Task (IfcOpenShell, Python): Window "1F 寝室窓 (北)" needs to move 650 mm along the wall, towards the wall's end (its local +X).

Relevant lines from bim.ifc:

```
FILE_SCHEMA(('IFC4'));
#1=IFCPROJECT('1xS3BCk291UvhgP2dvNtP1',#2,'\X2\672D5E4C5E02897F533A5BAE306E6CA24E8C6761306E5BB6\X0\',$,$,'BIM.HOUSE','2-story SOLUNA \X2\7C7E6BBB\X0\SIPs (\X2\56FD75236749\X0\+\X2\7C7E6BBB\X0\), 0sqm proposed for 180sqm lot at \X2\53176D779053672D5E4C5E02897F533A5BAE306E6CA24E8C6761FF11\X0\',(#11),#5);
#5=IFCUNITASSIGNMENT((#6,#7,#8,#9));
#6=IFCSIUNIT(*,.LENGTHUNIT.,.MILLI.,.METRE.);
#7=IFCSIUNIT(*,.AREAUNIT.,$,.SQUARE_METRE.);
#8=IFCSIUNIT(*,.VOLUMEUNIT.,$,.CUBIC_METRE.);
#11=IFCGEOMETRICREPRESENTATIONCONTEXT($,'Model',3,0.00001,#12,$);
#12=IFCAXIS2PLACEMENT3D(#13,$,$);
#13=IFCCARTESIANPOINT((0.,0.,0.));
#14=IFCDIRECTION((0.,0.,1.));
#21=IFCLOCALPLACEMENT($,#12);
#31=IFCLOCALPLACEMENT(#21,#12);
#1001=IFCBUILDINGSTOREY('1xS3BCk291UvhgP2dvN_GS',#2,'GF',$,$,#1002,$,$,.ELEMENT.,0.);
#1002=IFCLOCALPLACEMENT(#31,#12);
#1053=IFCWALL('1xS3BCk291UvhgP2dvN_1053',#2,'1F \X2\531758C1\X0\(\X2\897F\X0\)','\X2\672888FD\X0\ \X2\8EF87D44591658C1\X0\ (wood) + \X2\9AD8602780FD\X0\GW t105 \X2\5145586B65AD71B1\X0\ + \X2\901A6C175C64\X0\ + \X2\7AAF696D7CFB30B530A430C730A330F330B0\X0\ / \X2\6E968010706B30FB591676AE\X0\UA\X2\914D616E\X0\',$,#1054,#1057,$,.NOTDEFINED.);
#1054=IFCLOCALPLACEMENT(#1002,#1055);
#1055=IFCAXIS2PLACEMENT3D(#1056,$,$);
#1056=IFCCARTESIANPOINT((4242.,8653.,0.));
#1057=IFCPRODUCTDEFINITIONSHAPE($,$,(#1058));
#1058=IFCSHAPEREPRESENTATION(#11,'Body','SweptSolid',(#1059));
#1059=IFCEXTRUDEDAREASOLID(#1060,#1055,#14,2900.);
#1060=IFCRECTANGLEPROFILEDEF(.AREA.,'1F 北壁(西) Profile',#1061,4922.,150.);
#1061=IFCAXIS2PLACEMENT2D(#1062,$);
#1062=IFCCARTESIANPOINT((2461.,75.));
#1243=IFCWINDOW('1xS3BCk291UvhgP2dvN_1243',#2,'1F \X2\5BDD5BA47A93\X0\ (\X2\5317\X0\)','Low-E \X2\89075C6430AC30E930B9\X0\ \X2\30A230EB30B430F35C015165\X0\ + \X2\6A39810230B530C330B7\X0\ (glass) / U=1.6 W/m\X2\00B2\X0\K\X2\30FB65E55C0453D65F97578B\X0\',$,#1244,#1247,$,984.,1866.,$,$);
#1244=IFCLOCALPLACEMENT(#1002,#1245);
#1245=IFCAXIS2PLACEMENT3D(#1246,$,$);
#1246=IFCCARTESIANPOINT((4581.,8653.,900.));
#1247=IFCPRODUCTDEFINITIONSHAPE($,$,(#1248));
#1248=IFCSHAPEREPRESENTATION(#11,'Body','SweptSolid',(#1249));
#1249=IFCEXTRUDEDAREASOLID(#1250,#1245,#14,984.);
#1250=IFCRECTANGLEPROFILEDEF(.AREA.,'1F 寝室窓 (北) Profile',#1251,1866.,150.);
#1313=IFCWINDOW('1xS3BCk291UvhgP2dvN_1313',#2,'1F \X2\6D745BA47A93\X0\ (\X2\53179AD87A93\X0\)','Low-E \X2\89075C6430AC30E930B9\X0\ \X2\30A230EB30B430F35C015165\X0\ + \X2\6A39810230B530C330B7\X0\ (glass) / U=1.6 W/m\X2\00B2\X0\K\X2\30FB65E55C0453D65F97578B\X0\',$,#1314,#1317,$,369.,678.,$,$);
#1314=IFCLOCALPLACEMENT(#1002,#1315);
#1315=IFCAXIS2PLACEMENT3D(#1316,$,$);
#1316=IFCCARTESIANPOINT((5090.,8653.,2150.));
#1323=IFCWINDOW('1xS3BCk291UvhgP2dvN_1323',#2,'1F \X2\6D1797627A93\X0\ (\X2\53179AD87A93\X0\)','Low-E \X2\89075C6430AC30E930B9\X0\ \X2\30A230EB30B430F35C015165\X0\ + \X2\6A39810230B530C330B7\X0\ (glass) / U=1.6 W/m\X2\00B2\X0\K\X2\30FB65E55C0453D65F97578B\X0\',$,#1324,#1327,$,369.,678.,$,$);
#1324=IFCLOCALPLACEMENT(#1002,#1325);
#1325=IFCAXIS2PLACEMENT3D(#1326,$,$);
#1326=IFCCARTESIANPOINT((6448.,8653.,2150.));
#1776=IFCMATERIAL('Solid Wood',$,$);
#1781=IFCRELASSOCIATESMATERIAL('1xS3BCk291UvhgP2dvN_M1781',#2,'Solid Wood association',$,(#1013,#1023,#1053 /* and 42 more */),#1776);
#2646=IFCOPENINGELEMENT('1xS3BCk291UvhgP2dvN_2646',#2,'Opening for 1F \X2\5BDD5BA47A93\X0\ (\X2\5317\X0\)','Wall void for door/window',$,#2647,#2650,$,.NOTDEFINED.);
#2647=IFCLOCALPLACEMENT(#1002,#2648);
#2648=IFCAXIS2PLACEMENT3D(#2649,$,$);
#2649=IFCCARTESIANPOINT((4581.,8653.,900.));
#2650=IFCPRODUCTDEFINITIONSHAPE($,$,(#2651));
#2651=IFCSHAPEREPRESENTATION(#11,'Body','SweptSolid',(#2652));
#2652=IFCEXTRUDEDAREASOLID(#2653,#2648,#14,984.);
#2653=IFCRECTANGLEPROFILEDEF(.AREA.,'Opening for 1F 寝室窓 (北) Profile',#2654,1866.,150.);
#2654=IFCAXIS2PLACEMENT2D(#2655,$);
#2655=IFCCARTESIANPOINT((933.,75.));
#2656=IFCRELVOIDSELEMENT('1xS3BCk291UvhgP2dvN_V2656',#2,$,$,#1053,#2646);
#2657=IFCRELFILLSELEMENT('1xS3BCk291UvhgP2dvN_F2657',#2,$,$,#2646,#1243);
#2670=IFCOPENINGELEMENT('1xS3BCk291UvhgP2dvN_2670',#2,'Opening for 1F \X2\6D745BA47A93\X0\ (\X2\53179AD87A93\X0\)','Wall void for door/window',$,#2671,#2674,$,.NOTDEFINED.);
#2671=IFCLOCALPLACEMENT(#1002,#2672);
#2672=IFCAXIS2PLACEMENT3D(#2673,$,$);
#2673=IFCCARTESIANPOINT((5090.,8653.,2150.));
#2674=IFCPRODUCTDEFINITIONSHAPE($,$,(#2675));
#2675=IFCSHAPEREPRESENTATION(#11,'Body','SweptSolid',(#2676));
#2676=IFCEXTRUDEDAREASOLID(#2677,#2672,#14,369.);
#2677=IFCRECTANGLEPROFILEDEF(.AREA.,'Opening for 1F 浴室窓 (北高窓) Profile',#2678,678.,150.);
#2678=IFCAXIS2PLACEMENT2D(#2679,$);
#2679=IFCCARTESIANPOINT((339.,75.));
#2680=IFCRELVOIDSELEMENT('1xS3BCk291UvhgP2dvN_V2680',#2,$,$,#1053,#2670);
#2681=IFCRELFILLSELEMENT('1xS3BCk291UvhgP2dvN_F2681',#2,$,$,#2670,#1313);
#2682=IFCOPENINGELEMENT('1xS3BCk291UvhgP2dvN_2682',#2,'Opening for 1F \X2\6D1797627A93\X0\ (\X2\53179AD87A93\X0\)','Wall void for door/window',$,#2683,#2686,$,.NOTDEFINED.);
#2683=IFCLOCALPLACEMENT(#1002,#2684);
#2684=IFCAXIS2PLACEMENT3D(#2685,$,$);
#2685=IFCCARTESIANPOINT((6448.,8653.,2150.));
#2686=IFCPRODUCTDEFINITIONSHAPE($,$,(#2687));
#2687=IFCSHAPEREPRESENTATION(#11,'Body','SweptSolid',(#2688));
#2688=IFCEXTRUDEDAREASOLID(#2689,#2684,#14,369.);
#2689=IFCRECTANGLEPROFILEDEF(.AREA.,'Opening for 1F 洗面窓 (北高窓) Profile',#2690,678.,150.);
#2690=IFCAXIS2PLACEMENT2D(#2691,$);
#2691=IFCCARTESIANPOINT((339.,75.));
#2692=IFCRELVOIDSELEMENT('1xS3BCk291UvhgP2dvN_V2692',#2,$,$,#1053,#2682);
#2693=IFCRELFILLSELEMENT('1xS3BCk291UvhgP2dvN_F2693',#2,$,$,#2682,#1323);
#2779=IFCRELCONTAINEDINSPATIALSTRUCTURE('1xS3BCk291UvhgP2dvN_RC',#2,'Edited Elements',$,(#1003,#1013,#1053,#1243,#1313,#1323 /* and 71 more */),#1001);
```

```python
import ifcopenshell
import ifcopenshell.api.geometry
import ifcopenshell.util.placement
import ifcopenshell.util.unit

model = ifcopenshell.open("bim.ifc")
unit_scale = ifcopenshell.util.unit.calculate_unit_scale(model)

window = model.by_guid("1xS3BCk291UvhgP2dvN_1243")
opening = window.FillsVoids[0].RelatingOpeningElement
wall = opening.VoidsElements[0].RelatingBuildingElement

wall_matrix = ifcopenshell.util.placement.get_local_placement(wall.ObjectPlacement)
shift = wall_matrix[:3, 0] * 0.65 / unit_scale
before = ifcopenshell.util.placement.get_local_placement(window.ObjectPlacement)[:3, 3].copy()

# The window is not placed relative to its opening, so move both.
for product in (opening, window):
    matrix = ifcopenshell.util.placement.get_local_placement(product.ObjectPlacement)
    matrix[:3, 3] += shift
    ifcopenshell.api.geometry.edit_object_placement(model, product=product, matrix=matrix, is_si=False)

after = ifcopenshell.util.placement.get_local_placement(window.ObjectPlacement)[:3, 3]
print("window moved by", (after - before).round(3) + 0.0)

model.write("bim_updated.ifc")
```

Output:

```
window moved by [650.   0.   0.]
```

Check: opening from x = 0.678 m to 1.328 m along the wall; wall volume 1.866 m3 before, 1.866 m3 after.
